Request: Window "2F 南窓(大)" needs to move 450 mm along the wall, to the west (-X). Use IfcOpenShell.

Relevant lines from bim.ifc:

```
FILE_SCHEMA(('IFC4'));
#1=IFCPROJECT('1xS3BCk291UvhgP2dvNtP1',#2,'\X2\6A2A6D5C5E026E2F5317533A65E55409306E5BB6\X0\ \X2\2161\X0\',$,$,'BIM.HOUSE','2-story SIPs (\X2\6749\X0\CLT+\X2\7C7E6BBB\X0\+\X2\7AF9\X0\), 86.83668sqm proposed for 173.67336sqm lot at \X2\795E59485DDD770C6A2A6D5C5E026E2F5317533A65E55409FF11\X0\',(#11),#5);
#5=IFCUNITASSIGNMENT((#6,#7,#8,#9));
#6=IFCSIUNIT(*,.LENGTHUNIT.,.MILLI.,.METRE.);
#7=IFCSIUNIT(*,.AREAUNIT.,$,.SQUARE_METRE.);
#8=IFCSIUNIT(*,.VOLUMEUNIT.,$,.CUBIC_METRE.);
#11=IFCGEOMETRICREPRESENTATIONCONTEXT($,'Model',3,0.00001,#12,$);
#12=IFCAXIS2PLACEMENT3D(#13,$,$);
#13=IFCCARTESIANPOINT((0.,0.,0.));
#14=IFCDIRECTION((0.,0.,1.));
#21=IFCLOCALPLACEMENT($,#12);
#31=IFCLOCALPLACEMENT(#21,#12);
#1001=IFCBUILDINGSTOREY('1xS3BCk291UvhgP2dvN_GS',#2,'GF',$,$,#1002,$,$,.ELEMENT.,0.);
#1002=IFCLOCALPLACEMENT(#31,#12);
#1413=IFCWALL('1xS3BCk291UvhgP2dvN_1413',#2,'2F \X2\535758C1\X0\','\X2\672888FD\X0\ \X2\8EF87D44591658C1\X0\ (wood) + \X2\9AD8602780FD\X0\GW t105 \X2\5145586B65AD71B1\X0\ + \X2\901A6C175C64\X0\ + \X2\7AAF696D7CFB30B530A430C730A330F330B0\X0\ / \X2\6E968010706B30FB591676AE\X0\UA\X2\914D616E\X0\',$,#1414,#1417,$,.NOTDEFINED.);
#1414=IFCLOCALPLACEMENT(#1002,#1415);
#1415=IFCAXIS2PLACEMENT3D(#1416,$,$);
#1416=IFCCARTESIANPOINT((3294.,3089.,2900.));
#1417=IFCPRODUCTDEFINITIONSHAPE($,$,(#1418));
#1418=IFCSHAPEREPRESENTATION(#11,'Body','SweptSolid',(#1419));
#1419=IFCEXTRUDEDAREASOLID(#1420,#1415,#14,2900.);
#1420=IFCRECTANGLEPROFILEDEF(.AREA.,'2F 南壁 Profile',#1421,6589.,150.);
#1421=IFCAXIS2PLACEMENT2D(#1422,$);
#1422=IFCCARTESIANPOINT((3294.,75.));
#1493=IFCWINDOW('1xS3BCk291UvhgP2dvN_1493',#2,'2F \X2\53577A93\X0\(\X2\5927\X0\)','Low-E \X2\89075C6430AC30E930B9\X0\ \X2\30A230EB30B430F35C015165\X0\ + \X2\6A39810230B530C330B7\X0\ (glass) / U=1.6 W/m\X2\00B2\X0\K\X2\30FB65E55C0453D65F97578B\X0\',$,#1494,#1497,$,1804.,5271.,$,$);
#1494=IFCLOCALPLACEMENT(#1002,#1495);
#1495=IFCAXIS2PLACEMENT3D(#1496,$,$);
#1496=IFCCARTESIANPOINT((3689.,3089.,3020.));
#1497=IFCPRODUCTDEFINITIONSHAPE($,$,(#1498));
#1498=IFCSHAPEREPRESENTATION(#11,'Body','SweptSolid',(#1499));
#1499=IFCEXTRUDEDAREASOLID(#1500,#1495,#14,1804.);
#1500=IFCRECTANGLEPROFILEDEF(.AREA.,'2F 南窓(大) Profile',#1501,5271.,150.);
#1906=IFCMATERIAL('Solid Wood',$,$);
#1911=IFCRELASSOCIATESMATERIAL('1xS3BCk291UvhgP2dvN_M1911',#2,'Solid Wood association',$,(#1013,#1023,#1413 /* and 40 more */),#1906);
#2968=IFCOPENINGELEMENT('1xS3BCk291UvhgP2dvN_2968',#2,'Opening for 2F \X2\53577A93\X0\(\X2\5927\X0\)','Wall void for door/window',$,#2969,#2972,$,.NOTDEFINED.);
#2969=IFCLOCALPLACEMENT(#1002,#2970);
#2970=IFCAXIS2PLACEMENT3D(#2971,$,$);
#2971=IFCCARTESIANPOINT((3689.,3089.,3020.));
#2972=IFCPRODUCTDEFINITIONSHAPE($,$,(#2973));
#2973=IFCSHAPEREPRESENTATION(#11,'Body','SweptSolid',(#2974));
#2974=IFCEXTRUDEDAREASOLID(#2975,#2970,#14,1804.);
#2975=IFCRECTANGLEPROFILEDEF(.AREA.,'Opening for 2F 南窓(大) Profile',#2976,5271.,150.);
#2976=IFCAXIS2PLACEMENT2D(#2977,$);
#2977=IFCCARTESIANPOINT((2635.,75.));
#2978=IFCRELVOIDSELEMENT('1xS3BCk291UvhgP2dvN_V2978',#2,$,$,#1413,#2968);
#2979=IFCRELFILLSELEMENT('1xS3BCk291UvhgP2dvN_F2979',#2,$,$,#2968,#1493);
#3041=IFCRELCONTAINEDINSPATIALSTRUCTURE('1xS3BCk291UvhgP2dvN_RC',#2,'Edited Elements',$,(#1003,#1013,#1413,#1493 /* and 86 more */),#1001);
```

```python
import ifcopenshell
import ifcopenshell.api.geometry
import ifcopenshell.util.placement
import ifcopenshell.util.unit

model = ifcopenshell.open("bim.ifc")
unit_scale = ifcopenshell.util.unit.calculate_unit_scale(model)

window = model.by_id(1493)
opening = window.FillsVoids[0].RelatingOpeningElement
wall = opening.VoidsElements[0].RelatingBuildingElement

wall_matrix = ifcopenshell.util.placement.get_local_placement(wall.ObjectPlacement)
shift = wall_matrix[:3, 0] * -0.45 / unit_scale
before = ifcopenshell.util.placement.get_local_placement(window.ObjectPlacement)[:3, 3].copy()

# The window is not placed relative to its opening, so move both.
for product in (opening, window):
    matrix = ifcopenshell.util.placement.get_local_placement(product.ObjectPlacement)
    matrix[:3, 3] += shift
    ifcopenshell.api.geometry.edit_object_placement(model, product=product, matrix=matrix, is_si=False)

after = ifcopenshell.util.placement.get_local_placement(window.ObjectPlacement)[:3, 3]
print("window moved by", (after - before).round(3) + 0.0)

model.write("bim-out.ifc")
```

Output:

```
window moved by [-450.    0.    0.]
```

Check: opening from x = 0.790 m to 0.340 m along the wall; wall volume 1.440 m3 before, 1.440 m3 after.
